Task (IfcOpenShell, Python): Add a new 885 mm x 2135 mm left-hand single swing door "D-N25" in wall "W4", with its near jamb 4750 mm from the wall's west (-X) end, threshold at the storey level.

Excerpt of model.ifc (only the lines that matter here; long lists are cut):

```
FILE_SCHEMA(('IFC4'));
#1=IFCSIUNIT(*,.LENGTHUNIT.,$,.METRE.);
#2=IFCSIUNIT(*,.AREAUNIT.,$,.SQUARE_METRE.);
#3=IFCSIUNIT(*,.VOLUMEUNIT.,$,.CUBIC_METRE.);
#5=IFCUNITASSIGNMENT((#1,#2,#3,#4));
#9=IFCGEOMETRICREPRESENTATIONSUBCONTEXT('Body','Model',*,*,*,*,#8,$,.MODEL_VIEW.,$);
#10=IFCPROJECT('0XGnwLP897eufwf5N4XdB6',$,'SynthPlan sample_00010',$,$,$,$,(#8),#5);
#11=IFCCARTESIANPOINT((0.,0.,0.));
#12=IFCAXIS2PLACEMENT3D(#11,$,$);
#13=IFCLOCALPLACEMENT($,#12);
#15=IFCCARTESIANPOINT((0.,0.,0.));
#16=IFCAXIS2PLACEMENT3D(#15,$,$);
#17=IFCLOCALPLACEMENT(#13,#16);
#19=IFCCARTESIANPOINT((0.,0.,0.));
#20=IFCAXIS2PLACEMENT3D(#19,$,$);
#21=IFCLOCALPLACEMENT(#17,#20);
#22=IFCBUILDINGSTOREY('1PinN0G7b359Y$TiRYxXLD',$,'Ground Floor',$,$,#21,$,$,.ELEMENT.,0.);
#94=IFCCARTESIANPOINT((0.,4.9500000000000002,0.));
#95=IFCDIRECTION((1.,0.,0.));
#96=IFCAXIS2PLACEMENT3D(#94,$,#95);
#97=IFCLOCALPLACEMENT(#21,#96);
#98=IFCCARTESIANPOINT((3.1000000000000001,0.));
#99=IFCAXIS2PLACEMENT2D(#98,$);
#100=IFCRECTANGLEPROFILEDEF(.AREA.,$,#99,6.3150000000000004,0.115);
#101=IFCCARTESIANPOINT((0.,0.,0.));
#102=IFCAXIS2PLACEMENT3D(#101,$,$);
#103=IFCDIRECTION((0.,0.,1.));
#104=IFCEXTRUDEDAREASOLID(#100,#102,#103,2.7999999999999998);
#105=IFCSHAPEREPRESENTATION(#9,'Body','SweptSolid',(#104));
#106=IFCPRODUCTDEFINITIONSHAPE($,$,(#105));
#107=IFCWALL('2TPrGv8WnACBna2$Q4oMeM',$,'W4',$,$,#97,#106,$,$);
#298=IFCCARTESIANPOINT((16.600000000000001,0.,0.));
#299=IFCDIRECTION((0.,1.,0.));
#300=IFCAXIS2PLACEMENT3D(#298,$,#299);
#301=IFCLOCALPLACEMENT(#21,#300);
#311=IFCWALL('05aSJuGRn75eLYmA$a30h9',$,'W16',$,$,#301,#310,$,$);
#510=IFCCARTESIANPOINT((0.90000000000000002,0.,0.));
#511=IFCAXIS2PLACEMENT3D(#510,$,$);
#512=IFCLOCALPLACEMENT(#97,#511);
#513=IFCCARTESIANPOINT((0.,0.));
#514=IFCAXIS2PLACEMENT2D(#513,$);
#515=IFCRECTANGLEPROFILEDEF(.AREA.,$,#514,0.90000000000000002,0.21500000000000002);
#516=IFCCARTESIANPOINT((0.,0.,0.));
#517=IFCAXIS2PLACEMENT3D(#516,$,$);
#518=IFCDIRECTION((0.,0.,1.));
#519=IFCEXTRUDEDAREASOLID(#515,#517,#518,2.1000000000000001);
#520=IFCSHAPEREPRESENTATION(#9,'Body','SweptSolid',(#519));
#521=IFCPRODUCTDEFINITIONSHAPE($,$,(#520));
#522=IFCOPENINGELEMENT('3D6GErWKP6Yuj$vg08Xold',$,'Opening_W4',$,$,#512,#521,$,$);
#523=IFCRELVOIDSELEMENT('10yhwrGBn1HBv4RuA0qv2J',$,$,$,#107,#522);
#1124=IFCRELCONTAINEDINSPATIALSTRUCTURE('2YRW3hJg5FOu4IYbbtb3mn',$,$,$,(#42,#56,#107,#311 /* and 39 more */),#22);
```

```python
import numpy as np
import ifcopenshell
import ifcopenshell.api.feature
import ifcopenshell.api.geometry
import ifcopenshell.api.root
import ifcopenshell.api.spatial
import ifcopenshell.geom
import ifcopenshell.util.element
import ifcopenshell.util.placement
import ifcopenshell.util.representation
import ifcopenshell.util.shape
import ifcopenshell.util.unit

model = ifcopenshell.open("model.ifc")
unit_scale = ifcopenshell.util.unit.calculate_unit_scale(model)
settings = ifcopenshell.geom.settings()


def volume(element):
    """Net volume in cubic metres, openings subtracted."""
    shape = ifcopenshell.geom.create_shape(settings, element)
    return ifcopenshell.util.shape.get_volume(shape.geometry)


wall = model.by_guid("2TPrGv8WnACBna2$Q4oMeM")
storey = ifcopenshell.util.element.get_container(wall, ifc_class="IfcBuildingStorey")
context = ifcopenshell.util.representation.get_context(model, "Model", "Body", "MODEL_VIEW")
before = volume(wall)

width, height, from_end, sill = 0.885, 2.135, 4.75, 0.0  # metres

# The wall runs along its own X axis, and the end named is its -X end.
wall_shape = ifcopenshell.geom.create_shape(settings, wall)
x, y, z = ifcopenshell.util.shape.get_vertices(wall_shape.geometry).T
start = x.min() + from_end
face, thickness = float(y.min()), float(y.max() - y.min())
wall_matrix = ifcopenshell.util.placement.get_local_placement(wall.ObjectPlacement)
level = ifcopenshell.util.placement.get_local_placement(storey.ObjectPlacement)[2, 3]


def in_wall(x, y):
    """Placement at x, y metres in the wall's axes, at sill height."""
    matrix = wall_matrix.copy()
    matrix[:, 3] = wall_matrix @ np.array([x / unit_scale, y / unit_scale, 0.0, 1.0])
    matrix[2, 3] = level + sill / unit_scale
    return matrix


# Opening: a box that overshoots both wall faces by 50 mm.
opening = ifcopenshell.api.root.create_entity(model, ifc_class="IfcOpeningElement", predefined_type="OPENING")
box = ifcopenshell.api.geometry.add_wall_representation(
    model, context=context, length=width, height=height, thickness=thickness + 0.1
)
ifcopenshell.api.geometry.assign_representation(model, product=opening, representation=box)
ifcopenshell.api.geometry.edit_object_placement(model, product=opening, matrix=in_wall(start, face - 0.05), is_si=False)
ifcopenshell.api.feature.add_feature(model, feature=opening, element=wall)

door = ifcopenshell.api.root.create_entity(model, ifc_class="IfcDoor", name="D-N25", predefined_type="DOOR")
door.OverallWidth, door.OverallHeight = width / unit_scale, height / unit_scale
door.OperationType = "SINGLE_SWING_LEFT"
body = ifcopenshell.api.geometry.add_door_representation(
    model,
    context=context,
    overall_width=door.OverallWidth,
    overall_height=door.OverallHeight,
    operation_type="SINGLE_SWING_LEFT",
    lining_properties={"LiningDepth": thickness / unit_scale, "ThresholdDepth": thickness / unit_scale},
)
ifcopenshell.api.geometry.assign_representation(model, product=door, representation=body)
ifcopenshell.api.spatial.assign_container(model, products=[door], relating_structure=storey)
ifcopenshell.api.feature.add_filling(model, opening=opening, element=door)

# The lining spans the wall, so the door starts at the wall face.
ifcopenshell.api.geometry.edit_object_placement(model, product=door, matrix=in_wall(start, face), is_si=False)

after = volume(wall)

print(f"wall volume {before:.3f} -> {after:.3f} m3")

model.write("model_edited.ifc")
```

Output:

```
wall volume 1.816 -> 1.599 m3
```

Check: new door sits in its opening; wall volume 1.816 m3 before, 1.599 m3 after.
